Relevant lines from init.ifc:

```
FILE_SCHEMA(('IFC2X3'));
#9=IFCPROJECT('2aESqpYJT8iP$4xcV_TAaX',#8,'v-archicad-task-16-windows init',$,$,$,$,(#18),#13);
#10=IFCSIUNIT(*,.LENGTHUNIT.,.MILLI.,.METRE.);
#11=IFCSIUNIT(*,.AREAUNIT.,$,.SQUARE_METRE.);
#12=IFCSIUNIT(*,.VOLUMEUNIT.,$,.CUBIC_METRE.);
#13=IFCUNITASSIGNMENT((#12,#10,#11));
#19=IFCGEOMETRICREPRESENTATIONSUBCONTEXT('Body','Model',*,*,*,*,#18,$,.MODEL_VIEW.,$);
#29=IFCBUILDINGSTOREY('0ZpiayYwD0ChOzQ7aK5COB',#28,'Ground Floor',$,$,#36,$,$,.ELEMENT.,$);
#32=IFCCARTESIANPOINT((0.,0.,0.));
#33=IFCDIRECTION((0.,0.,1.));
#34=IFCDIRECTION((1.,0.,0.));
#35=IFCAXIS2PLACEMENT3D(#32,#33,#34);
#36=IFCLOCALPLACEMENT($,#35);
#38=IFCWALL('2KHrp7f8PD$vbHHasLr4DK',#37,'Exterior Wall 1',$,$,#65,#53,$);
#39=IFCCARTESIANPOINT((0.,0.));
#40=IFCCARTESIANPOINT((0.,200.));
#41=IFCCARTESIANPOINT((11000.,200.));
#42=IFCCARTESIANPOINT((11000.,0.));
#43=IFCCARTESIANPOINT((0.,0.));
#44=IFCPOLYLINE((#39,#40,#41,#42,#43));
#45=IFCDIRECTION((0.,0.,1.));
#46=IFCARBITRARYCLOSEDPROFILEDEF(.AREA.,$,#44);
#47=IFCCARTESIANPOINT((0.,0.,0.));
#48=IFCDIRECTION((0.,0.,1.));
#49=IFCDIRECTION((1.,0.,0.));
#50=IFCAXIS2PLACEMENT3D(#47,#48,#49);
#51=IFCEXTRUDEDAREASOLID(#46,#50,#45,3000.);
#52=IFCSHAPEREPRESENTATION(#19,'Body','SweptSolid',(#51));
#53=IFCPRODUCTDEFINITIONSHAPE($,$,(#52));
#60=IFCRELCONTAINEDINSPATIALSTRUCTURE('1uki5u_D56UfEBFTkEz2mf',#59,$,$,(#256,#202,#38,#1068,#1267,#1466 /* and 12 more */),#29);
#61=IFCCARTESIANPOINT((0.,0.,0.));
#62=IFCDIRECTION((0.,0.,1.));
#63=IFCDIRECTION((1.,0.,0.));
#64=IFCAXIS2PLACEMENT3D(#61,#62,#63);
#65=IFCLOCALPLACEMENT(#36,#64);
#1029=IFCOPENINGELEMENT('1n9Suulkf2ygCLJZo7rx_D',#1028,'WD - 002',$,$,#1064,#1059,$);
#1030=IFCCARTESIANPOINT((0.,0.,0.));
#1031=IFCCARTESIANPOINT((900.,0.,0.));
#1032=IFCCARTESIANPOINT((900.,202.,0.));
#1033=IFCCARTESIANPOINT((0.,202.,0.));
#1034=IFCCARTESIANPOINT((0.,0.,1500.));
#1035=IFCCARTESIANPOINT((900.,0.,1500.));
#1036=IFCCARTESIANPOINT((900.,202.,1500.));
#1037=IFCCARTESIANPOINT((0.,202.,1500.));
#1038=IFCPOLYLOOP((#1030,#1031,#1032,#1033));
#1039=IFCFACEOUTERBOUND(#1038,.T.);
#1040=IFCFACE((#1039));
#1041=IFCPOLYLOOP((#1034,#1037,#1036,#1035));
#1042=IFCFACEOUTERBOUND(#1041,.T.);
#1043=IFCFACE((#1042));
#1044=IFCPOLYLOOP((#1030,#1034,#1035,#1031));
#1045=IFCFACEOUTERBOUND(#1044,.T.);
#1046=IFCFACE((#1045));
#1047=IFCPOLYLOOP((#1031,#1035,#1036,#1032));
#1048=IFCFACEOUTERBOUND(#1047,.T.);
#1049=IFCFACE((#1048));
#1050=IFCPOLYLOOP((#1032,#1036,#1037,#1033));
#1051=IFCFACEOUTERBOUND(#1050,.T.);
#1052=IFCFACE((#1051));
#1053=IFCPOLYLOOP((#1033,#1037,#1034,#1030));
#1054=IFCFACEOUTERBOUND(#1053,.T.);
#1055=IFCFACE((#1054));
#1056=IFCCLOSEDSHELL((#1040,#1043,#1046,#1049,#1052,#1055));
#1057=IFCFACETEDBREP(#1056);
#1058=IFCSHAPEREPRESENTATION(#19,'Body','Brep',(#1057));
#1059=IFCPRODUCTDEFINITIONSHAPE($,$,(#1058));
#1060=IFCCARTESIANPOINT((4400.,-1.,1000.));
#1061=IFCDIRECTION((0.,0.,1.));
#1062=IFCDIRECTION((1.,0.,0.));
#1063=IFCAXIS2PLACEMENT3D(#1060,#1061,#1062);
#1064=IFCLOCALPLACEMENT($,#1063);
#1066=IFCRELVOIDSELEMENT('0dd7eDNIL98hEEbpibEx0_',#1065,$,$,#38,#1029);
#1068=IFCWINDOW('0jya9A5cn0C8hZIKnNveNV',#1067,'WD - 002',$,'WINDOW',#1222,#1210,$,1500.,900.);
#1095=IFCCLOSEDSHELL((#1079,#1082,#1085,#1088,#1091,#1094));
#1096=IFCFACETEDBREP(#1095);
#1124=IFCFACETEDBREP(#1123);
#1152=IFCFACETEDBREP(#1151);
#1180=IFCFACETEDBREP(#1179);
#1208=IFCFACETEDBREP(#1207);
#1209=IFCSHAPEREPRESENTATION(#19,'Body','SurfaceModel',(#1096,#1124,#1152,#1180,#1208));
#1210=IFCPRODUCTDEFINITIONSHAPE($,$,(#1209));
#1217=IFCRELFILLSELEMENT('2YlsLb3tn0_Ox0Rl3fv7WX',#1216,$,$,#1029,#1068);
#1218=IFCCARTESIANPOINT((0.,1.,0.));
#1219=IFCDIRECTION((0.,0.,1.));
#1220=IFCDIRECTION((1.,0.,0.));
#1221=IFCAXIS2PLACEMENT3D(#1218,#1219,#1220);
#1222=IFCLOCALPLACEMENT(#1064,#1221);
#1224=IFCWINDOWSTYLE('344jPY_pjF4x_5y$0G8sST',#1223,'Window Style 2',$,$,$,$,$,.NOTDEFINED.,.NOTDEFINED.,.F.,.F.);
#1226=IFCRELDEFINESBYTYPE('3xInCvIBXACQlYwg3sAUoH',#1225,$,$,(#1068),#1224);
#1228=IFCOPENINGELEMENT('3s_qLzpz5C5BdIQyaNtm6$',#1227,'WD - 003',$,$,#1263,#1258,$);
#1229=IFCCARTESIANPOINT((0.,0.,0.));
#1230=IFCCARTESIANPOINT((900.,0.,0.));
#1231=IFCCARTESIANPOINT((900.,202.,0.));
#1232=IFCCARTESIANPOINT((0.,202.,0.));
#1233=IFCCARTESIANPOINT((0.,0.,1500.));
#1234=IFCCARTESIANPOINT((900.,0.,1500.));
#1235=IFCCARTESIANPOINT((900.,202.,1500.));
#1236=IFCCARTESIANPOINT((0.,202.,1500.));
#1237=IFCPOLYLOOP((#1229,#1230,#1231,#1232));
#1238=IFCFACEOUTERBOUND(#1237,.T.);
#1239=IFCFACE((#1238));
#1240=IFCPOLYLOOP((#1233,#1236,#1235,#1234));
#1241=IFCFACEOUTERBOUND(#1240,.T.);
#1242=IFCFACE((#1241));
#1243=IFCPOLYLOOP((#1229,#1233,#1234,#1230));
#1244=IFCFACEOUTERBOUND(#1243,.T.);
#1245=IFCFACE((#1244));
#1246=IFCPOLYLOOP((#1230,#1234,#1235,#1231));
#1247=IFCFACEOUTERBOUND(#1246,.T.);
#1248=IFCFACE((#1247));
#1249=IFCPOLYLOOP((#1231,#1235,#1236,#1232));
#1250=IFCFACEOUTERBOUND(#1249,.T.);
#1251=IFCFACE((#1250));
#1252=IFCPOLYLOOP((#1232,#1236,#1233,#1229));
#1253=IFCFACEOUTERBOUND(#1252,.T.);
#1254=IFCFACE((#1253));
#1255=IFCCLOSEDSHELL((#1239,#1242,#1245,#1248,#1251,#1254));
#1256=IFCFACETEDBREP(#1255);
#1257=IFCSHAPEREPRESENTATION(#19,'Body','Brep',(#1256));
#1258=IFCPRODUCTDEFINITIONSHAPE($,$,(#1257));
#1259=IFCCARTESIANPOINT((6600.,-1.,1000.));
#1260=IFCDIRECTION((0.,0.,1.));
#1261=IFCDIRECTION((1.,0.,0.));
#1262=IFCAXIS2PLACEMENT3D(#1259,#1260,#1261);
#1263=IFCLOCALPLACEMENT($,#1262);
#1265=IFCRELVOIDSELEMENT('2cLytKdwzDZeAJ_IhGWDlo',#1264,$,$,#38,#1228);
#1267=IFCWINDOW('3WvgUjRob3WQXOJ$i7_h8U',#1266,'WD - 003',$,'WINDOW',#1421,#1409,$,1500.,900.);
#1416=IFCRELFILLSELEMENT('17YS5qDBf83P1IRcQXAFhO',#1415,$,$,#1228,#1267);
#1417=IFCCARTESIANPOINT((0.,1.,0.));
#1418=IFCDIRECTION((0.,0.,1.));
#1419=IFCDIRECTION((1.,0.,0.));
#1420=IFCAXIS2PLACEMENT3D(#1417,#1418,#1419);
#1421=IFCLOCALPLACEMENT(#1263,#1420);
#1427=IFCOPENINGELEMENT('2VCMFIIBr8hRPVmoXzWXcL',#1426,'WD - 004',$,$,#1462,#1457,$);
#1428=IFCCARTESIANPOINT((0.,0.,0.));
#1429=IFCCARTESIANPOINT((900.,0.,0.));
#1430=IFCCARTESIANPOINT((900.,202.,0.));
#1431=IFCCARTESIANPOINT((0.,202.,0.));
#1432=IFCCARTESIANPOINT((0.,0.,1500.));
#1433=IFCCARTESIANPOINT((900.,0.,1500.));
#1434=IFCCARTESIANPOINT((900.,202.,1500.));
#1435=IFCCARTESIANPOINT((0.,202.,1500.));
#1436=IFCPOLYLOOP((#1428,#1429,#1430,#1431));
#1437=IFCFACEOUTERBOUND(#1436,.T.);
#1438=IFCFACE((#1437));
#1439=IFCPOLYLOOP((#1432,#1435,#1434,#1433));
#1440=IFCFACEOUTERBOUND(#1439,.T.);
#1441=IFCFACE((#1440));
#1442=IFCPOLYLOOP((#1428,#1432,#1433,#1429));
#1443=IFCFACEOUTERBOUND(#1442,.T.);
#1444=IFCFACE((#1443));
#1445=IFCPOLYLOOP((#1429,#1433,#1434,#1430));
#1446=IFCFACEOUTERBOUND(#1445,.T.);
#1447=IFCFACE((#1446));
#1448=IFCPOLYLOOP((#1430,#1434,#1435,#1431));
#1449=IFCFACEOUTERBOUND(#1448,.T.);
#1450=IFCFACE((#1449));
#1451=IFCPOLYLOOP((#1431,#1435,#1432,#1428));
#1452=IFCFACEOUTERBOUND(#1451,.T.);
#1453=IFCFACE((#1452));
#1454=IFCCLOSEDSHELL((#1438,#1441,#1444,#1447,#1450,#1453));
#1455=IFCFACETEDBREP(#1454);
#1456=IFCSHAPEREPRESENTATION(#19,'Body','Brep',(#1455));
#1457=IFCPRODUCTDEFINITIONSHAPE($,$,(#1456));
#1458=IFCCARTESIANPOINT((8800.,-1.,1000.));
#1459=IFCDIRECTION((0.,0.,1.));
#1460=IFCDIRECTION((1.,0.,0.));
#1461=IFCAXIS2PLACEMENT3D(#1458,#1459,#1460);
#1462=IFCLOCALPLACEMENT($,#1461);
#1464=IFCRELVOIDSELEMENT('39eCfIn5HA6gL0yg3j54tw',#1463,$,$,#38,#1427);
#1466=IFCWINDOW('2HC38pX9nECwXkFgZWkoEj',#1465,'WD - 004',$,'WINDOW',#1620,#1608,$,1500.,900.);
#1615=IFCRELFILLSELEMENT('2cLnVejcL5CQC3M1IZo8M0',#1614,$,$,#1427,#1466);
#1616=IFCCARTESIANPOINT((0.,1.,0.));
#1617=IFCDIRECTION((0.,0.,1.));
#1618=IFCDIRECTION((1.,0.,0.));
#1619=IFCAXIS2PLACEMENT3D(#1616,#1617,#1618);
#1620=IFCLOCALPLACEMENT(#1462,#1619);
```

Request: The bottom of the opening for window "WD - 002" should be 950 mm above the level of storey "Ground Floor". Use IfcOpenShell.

```python
import numpy as np
import ifcopenshell
import ifcopenshell.api.geometry
import ifcopenshell.geom
import ifcopenshell.util.element
import ifcopenshell.util.placement
import ifcopenshell.util.shape
import ifcopenshell.util.unit

model = ifcopenshell.open("init.ifc")
unit_scale = ifcopenshell.util.unit.calculate_unit_scale(model)

window = model.by_guid("0jya9A5cn0C8hZIKnNveNV")
opening = window.FillsVoids[0].RelatingOpeningElement
storey = ifcopenshell.util.element.get_container(window, ifc_class="IfcBuildingStorey")
level = ifcopenshell.util.placement.get_local_placement(storey.ObjectPlacement)[2, 3]

# The opening's origin need not be at the sill, so measure its lowest point.
shape = ifcopenshell.geom.create_shape(ifcopenshell.geom.settings(), opening)
bottom = ifcopenshell.util.shape.get_shape_bottom_elevation(shape, shape.geometry) / unit_scale
dz = level + 0.95 / unit_scale - bottom

shift = np.array([0.0, 0.0, dz])
# The window is placed relative to its opening, so it follows when the opening moves.
matrix = ifcopenshell.util.placement.get_local_placement(opening.ObjectPlacement)
matrix[:3, 3] += shift
ifcopenshell.api.geometry.edit_object_placement(
    model, product=opening, matrix=matrix, is_si=False, should_transform_children=True
)

print(f"moved by {dz * unit_scale:+.3f} m")

model.write("init_rev.ifc")
```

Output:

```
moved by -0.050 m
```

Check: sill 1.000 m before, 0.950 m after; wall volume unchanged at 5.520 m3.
